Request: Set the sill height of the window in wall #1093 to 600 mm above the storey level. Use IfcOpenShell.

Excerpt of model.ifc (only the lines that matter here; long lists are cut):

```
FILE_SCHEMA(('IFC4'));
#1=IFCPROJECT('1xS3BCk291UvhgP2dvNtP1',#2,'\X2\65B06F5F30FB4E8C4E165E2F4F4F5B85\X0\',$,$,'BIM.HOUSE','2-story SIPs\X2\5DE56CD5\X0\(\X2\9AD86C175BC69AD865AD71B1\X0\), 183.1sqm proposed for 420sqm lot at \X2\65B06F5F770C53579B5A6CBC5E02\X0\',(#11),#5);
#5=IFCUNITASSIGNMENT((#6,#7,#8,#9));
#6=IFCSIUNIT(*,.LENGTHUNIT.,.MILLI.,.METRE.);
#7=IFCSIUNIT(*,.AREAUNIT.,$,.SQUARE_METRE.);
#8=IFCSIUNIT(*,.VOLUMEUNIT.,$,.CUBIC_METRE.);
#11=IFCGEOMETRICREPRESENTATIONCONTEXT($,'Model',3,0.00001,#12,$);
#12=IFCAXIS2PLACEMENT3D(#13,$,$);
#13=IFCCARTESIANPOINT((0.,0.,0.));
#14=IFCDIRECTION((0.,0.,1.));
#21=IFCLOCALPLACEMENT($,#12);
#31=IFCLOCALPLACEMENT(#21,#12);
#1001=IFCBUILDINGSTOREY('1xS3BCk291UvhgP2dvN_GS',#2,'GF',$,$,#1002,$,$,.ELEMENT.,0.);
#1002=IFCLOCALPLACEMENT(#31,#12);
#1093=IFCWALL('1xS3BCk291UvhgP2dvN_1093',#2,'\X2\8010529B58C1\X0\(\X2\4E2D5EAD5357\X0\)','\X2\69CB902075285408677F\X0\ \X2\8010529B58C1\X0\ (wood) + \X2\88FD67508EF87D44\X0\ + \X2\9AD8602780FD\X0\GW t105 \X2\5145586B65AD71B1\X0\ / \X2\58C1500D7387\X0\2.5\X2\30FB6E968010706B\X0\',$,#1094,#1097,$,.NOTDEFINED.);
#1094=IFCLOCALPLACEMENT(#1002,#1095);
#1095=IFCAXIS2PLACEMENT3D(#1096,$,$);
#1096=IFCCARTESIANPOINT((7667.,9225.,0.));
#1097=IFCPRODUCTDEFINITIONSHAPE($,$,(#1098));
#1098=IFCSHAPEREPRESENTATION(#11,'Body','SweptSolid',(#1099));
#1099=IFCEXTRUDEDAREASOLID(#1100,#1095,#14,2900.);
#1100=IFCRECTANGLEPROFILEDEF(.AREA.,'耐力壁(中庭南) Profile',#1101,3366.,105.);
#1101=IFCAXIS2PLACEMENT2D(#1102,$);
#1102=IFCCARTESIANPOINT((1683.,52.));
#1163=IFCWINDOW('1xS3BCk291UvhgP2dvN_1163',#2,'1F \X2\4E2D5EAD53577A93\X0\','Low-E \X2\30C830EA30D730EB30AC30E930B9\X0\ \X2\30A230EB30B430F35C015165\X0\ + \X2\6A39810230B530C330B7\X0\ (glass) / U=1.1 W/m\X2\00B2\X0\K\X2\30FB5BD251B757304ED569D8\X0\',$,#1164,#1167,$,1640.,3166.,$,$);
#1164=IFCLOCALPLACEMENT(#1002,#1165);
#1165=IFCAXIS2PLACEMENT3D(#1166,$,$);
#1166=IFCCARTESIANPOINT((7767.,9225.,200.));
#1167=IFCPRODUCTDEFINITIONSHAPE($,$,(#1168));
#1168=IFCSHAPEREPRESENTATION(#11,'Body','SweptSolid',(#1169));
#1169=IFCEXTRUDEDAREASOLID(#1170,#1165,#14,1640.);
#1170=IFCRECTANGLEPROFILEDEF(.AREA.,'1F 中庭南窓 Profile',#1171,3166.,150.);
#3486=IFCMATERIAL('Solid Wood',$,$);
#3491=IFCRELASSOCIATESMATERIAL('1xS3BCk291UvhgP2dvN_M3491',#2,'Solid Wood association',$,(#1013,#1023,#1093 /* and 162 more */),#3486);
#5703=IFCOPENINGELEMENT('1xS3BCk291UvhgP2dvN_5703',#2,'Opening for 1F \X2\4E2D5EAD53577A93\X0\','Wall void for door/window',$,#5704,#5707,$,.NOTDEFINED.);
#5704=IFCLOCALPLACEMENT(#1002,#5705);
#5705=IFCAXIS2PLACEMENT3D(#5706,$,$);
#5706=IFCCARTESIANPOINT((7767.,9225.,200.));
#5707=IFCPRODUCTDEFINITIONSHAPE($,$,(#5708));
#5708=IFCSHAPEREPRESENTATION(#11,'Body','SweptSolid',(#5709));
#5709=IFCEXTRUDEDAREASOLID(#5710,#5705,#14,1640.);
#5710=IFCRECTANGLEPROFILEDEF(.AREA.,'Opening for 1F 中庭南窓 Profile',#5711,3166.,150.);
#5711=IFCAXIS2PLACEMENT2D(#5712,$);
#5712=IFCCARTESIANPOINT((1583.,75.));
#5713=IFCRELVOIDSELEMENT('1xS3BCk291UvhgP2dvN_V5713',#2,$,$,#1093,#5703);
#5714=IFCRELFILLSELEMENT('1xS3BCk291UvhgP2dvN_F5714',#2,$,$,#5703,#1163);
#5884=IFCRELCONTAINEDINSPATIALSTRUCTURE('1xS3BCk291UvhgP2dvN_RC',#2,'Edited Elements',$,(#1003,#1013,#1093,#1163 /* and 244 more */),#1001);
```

```python
import numpy as np
import ifcopenshell
import ifcopenshell.api.geometry
import ifcopenshell.geom
import ifcopenshell.util.element
import ifcopenshell.util.placement
import ifcopenshell.util.shape
import ifcopenshell.util.unit

model = ifcopenshell.open("model.ifc")
unit_scale = ifcopenshell.util.unit.calculate_unit_scale(model)

window = model.by_guid("1xS3BCk291UvhgP2dvN_1163")
opening = window.FillsVoids[0].RelatingOpeningElement
storey = ifcopenshell.util.element.get_container(window, ifc_class="IfcBuildingStorey")
level = ifcopenshell.util.placement.get_local_placement(storey.ObjectPlacement)[2, 3]

# The opening's origin need not be at the sill, so measure its lowest point.
shape = ifcopenshell.geom.create_shape(ifcopenshell.geom.settings(), opening)
bottom = ifcopenshell.util.shape.get_shape_bottom_elevation(shape, shape.geometry) / unit_scale
dz = level + 0.6 / unit_scale - bottom

shift = np.array([0.0, 0.0, dz])
# The window is not placed relative to its opening, so move both.
for product in (opening, window):
    matrix = ifcopenshell.util.placement.get_local_placement(product.ObjectPlacement)
    matrix[:3, 3] += shift
    ifcopenshell.api.geometry.edit_object_placement(model, product=product, matrix=matrix, is_si=False)

print(f"moved by {dz * unit_scale:+.3f} m")

model.write("model_rev.ifc")
```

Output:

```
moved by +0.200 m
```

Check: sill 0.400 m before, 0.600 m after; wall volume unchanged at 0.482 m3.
